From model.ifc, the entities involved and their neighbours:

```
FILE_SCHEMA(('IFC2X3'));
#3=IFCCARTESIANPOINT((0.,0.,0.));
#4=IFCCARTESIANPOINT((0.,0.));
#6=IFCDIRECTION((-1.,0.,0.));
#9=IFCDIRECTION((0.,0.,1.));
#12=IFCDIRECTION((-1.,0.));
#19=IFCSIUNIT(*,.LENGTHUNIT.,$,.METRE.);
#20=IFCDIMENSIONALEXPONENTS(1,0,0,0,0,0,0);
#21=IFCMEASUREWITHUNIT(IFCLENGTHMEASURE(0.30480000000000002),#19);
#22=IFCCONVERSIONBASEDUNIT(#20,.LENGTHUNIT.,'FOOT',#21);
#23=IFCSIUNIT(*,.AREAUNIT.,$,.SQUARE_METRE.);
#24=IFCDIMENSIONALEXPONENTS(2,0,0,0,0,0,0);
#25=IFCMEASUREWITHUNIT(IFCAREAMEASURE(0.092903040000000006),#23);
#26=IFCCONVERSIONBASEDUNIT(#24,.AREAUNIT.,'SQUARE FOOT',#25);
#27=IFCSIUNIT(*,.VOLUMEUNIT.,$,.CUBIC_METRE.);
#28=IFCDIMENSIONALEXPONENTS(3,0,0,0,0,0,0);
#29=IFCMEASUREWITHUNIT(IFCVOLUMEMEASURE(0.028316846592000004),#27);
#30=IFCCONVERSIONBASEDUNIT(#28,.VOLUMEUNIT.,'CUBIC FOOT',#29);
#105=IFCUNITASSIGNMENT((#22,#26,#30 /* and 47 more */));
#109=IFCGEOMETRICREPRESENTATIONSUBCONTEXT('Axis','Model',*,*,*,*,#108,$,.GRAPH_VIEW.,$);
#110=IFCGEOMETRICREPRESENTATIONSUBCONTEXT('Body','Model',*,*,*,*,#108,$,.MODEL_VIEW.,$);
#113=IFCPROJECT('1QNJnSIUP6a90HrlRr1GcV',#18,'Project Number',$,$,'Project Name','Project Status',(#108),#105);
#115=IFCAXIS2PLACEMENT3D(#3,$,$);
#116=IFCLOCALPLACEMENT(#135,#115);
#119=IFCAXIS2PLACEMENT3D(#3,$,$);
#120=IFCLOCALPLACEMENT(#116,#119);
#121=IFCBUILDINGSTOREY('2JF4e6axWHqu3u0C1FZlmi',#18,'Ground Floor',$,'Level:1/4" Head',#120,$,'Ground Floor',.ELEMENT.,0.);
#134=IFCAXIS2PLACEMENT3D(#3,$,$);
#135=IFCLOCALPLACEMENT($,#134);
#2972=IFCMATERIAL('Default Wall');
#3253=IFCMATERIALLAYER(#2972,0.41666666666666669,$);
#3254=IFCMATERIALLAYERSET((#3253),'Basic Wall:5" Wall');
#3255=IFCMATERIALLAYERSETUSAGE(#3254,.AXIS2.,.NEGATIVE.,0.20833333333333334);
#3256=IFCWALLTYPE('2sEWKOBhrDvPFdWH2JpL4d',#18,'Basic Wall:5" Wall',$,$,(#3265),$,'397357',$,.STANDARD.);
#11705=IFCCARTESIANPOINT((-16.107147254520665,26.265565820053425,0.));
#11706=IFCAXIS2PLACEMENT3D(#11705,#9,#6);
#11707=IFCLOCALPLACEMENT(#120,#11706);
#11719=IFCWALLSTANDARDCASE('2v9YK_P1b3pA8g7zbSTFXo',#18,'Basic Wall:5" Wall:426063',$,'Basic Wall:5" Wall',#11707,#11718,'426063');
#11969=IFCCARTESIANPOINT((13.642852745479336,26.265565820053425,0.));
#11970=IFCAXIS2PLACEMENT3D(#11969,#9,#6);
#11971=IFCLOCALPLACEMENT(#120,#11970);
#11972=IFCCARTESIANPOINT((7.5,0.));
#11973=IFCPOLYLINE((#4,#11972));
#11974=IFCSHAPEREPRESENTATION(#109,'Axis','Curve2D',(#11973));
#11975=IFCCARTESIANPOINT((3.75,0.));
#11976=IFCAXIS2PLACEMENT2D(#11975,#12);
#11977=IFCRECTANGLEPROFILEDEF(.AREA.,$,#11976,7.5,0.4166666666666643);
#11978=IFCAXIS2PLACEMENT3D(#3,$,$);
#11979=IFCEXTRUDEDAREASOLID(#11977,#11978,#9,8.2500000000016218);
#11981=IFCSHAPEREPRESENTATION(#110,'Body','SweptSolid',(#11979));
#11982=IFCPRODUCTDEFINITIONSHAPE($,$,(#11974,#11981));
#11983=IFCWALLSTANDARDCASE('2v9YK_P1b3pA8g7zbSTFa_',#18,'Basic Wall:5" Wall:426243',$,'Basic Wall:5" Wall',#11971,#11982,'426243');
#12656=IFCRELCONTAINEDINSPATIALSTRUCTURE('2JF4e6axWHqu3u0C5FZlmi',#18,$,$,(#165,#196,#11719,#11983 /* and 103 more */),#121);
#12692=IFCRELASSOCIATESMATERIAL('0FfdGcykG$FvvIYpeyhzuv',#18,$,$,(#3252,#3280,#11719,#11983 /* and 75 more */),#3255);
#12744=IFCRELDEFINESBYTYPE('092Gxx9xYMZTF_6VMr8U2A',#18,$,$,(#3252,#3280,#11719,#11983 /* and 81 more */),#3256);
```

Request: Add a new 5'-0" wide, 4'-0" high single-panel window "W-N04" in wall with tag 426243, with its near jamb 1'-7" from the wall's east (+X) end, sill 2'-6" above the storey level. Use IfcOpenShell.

```python
import numpy as np
import ifcopenshell
import ifcopenshell.api.feature
import ifcopenshell.api.geometry
import ifcopenshell.api.root
import ifcopenshell.api.spatial
import ifcopenshell.api.type
import ifcopenshell.geom
import ifcopenshell.util.element
import ifcopenshell.util.placement
import ifcopenshell.util.representation
import ifcopenshell.util.shape
import ifcopenshell.util.unit

model = ifcopenshell.open("model.ifc")
unit_scale = ifcopenshell.util.unit.calculate_unit_scale(model)
settings = ifcopenshell.geom.settings()


def volume(element):
    """Net volume in cubic metres, openings subtracted."""
    shape = ifcopenshell.geom.create_shape(settings, element)
    return ifcopenshell.util.shape.get_volume(shape.geometry)


wall = model.by_guid("2v9YK_P1b3pA8g7zbSTFa_")
storey = ifcopenshell.util.element.get_container(wall, ifc_class="IfcBuildingStorey")
context = ifcopenshell.util.representation.get_context(model, "Model", "Body", "MODEL_VIEW")
before = volume(wall)

width, height, from_end, sill = 1.524, 1.2192, 0.4826, 0.762  # metres

# The wall runs along its own X axis, and the end named is its -X end.
wall_shape = ifcopenshell.geom.create_shape(settings, wall)
x, y, z = ifcopenshell.util.shape.get_vertices(wall_shape.geometry).T
start = x.min() + from_end
face, thickness = float(y.min()), float(y.max() - y.min())
wall_matrix = ifcopenshell.util.placement.get_local_placement(wall.ObjectPlacement)
level = ifcopenshell.util.placement.get_local_placement(storey.ObjectPlacement)[2, 3]


def in_wall(x, y):
    """Placement at x, y metres in the wall's axes, at sill height."""
    matrix = wall_matrix.copy()
    matrix[:, 3] = wall_matrix @ np.array([x / unit_scale, y / unit_scale, 0.0, 1.0])
    matrix[2, 3] = level + sill / unit_scale
    return matrix


# Opening: a box that overshoots both wall faces by 50 mm.
opening = ifcopenshell.api.root.create_entity(model, ifc_class="IfcOpeningElement")
box = ifcopenshell.api.geometry.add_wall_representation(
    model, context=context, length=width, height=height, thickness=thickness + 0.1
)
ifcopenshell.api.geometry.assign_representation(model, product=opening, representation=box)
ifcopenshell.api.geometry.edit_object_placement(model, product=opening, matrix=in_wall(start, face - 0.05), is_si=False)
ifcopenshell.api.feature.add_feature(model, feature=opening, element=wall)

window = ifcopenshell.api.root.create_entity(model, ifc_class="IfcWindow", name="W-N04")
window.OverallWidth, window.OverallHeight = width / unit_scale, height / unit_scale
body = ifcopenshell.api.geometry.add_window_representation(
    model,
    context=context,
    overall_width=window.OverallWidth,
    overall_height=window.OverallHeight,
    partition_type="SINGLE_PANEL",
)
ifcopenshell.api.geometry.assign_representation(model, product=window, representation=body)
ifcopenshell.api.spatial.assign_container(model, products=[window], relating_structure=storey)
fills = ifcopenshell.api.feature.add_filling(model, opening=opening, element=window)
fills.OwnerHistory = window.OwnerHistory  # required in IFC2X3

# IFC2X3 keeps the operation on the window style.
style = ifcopenshell.api.root.create_entity(model, ifc_class="IfcWindowStyle", name="W-N04")
style.OperationType, style.ConstructionType = "SINGLE_PANEL", "NOTDEFINED"
style.ParameterTakesPrecedence = style.Sizeable = False
ifcopenshell.api.type.assign_type(model, related_objects=[window], relating_type=style)

# Centre the window in the wall's thickness.
ifcopenshell.api.geometry.edit_object_placement(model, product=window, matrix=in_wall(start, face), is_si=False)
window_shape = ifcopenshell.geom.create_shape(settings, window)
depth = ifcopenshell.util.shape.get_vertices(window_shape.geometry)[:, 1]
offset = face + thickness / 2 - (depth.min() + depth.max()) / 2
ifcopenshell.api.geometry.edit_object_placement(model, product=window, matrix=in_wall(start, offset), is_si=False)

after = volume(wall)

print(f"wall volume {before:.3f} -> {after:.3f} m3")

model.write("model_rev.ifc")
```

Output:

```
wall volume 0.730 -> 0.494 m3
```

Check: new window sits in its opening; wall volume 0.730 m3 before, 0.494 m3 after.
